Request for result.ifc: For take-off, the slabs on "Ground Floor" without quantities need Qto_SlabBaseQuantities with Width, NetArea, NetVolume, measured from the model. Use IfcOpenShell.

First a look at what the model holds.

```python
import ifcopenshell
import ifcopenshell.util.element
import ifcopenshell.util.unit

model = ifcopenshell.open("result.ifc")
print(model.schema)
for unit_type in ("LENGTHUNIT", "AREAUNIT", "VOLUMEUNIT"):
    print(unit_type, ifcopenshell.util.unit.calculate_unit_scale(model, unit_type))
storey = next(s for s in model.by_type("IfcBuildingStorey") if s.Name == "Ground Floor")
slabs = [e for e in ifcopenshell.util.element.get_decomposition(storey) if e.is_a("IfcSlab")]
for e in sorted(slabs, key=lambda e: e.id()):
    print(e.id(), e.is_a(), e.Name, list(ifcopenshell.util.element.get_psets(e, qtos_only=True)), sep=" | ")
```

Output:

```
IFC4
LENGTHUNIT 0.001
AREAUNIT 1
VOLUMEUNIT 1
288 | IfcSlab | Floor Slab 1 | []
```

```python
import ifcopenshell
import ifcopenshell.api.pset
import ifcopenshell.geom
import ifcopenshell.util.element
import ifcopenshell.util.shape
import ifcopenshell.util.unit

model = ifcopenshell.open("result.ifc")
unit_scale = ifcopenshell.util.unit.calculate_unit_scale(model)
area_scale = ifcopenshell.util.unit.calculate_unit_scale(model, "AREAUNIT")
volume_scale = ifcopenshell.util.unit.calculate_unit_scale(model, "VOLUMEUNIT")
settings = ifcopenshell.geom.settings()

storey = next(s for s in model.by_type("IfcBuildingStorey") if s.Name == "Ground Floor")
slabs = [e for e in ifcopenshell.util.element.get_decomposition(storey) if e.is_a("IfcSlab")]

for e in sorted(slabs, key=lambda e: e.id()):
    if ifcopenshell.util.element.get_psets(e, qtos_only=True, should_inherit=False):
        continue
    # Geometry comes back in metres, in the element's own axes.
    shape = ifcopenshell.geom.create_shape(settings, e)
    values = {
        "Width": ifcopenshell.util.shape.get_z(shape.geometry) / unit_scale,
        "NetArea": ifcopenshell.util.shape.get_footprint_area(shape.geometry) / area_scale,
        "NetVolume": ifcopenshell.util.shape.get_volume(shape.geometry) / volume_scale,
    }
    qto = ifcopenshell.api.pset.add_qto(model, product=e, name="Qto_SlabBaseQuantities")
    ifcopenshell.api.pset.edit_qto(model, qto=qto, properties=values)
    print(e.id(), {k: round(v, 3) for k, v in values.items()})

model.write("result_rev.ifc")
```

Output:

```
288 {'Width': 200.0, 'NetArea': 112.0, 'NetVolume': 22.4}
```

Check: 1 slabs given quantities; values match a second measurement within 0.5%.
